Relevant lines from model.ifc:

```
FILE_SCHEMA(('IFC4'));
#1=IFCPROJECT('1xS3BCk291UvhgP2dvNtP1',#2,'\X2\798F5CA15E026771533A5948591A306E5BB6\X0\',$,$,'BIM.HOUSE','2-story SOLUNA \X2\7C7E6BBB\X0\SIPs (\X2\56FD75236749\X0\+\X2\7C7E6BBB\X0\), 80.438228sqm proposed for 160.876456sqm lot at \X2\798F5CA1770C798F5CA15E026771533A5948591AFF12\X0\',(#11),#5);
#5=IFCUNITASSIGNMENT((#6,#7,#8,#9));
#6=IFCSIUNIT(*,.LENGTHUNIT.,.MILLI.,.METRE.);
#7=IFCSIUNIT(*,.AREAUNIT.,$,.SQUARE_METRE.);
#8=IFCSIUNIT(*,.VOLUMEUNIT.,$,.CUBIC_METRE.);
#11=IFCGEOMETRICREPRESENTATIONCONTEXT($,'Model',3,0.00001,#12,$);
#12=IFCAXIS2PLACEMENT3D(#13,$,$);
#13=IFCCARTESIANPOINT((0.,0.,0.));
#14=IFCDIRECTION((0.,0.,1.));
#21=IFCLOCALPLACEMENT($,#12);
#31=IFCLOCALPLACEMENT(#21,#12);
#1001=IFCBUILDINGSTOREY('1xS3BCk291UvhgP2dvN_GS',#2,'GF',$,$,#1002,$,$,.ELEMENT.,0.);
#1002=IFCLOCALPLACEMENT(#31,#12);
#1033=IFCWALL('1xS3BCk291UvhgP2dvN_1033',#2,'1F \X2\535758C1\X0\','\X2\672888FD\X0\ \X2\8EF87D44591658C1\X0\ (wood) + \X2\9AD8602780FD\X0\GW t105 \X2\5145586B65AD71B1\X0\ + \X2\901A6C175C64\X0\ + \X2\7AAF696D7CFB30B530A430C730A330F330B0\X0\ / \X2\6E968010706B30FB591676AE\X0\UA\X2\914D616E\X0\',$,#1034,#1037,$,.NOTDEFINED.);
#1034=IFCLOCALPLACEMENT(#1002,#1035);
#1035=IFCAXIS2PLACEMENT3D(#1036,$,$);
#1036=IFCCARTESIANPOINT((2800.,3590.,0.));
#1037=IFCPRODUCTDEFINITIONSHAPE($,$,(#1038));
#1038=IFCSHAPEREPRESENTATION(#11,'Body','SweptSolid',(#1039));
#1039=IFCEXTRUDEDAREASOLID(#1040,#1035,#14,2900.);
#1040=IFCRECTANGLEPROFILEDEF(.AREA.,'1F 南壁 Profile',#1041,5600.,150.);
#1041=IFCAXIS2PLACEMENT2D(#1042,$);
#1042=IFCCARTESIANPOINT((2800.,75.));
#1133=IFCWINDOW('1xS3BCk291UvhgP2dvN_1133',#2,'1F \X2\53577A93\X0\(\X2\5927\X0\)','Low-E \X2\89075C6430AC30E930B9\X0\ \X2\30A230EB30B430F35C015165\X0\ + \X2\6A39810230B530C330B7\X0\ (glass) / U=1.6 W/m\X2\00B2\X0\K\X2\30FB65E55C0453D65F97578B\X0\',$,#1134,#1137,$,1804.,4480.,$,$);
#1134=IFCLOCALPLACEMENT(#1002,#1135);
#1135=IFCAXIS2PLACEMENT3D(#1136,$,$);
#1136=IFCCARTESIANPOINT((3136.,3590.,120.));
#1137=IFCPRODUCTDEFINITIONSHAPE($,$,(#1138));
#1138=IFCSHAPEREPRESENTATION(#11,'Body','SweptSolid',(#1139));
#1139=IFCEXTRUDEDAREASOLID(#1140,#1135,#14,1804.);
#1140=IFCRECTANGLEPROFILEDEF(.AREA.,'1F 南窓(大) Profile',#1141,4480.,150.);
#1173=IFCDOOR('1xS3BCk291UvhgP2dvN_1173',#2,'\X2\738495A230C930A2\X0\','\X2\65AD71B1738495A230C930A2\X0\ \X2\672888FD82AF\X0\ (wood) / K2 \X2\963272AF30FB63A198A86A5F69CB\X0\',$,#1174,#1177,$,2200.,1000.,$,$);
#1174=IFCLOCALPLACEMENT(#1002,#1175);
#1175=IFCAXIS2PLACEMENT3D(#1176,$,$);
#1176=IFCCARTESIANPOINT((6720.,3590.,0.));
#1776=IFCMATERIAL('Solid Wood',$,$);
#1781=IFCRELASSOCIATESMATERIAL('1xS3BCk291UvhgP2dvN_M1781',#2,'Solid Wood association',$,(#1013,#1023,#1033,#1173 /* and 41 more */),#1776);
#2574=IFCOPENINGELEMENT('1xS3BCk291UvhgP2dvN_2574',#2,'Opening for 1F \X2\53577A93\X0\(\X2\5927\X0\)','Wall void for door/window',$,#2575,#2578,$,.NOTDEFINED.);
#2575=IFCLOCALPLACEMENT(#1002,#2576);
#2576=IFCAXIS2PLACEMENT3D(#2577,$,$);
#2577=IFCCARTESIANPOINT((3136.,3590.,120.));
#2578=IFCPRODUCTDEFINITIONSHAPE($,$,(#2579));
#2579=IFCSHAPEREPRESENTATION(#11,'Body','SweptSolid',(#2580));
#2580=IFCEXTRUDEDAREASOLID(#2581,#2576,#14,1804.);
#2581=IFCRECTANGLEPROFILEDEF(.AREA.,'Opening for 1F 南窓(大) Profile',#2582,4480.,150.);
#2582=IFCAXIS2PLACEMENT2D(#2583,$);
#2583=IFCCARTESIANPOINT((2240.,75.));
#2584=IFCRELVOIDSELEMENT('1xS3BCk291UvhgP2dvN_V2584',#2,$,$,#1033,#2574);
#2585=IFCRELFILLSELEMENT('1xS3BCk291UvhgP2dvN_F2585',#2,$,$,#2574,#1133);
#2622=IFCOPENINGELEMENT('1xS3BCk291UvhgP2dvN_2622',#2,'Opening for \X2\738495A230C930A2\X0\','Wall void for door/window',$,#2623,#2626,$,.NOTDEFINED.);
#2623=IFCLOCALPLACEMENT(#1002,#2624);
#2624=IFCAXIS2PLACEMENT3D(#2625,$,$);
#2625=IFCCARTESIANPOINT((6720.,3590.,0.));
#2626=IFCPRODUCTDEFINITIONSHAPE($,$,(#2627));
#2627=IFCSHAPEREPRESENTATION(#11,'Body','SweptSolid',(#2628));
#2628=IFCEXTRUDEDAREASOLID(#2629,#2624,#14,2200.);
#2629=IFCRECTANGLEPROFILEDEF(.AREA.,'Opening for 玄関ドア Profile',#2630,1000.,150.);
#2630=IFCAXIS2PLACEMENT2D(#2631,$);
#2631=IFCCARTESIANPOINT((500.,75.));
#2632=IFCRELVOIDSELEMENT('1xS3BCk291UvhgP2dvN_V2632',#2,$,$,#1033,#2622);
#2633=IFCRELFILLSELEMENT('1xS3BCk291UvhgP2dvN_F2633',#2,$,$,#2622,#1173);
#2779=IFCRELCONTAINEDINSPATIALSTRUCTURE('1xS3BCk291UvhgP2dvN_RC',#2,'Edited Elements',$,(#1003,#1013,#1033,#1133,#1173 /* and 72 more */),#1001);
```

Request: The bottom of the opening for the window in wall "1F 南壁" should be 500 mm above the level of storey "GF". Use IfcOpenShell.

```python
import numpy as np
import ifcopenshell
import ifcopenshell.api.geometry
import ifcopenshell.geom
import ifcopenshell.util.element
import ifcopenshell.util.placement
import ifcopenshell.util.shape
import ifcopenshell.util.unit

model = ifcopenshell.open("model.ifc")
unit_scale = ifcopenshell.util.unit.calculate_unit_scale(model)

window = model.by_id(1133)
opening = window.FillsVoids[0].RelatingOpeningElement
storey = ifcopenshell.util.element.get_container(window, ifc_class="IfcBuildingStorey")
level = ifcopenshell.util.placement.get_local_placement(storey.ObjectPlacement)[2, 3]

# The opening's origin need not be at the sill, so measure its lowest point.
shape = ifcopenshell.geom.create_shape(ifcopenshell.geom.settings(), opening)
bottom = ifcopenshell.util.shape.get_shape_bottom_elevation(shape, shape.geometry) / unit_scale
dz = level + 0.5 / unit_scale - bottom

shift = np.array([0.0, 0.0, dz])
# The window is not placed relative to its opening, so move both.
for product in (opening, window):
    matrix = ifcopenshell.util.placement.get_local_placement(product.ObjectPlacement)
    matrix[:3, 3] += shift
    ifcopenshell.api.geometry.edit_object_placement(model, product=product, matrix=matrix, is_si=False)

print(f"moved by {dz * unit_scale:+.3f} m")

model.write("model-out.ifc")
```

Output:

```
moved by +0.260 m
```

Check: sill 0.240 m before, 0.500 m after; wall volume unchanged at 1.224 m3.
